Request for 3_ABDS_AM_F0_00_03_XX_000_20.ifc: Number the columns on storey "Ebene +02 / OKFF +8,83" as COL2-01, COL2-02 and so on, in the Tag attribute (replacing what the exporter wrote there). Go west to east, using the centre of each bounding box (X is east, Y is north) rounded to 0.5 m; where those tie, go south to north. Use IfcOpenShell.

First a look at what the model holds.

```python
import ifcopenshell
import ifcopenshell.util.element
import ifcopenshell.util.placement

model = ifcopenshell.open("3_ABDS_AM_F0_00_03_XX_000_20.ifc")
print(model.schema)
storey = next(s for s in model.by_type("IfcBuildingStorey") if s.Name == "Ebene +02 / OKFF +8,83")
columns = [e for e in ifcopenshell.util.element.get_decomposition(storey) if e.is_a("IfcColumn")]
for e in sorted(columns, key=lambda e: e.id()):
    origin = ifcopenshell.util.placement.get_local_placement(e.ObjectPlacement)[:3, 3]
    print(e.id(), e.Tag, e.Name, origin.round(2) + 0.0, sep=" | ")
```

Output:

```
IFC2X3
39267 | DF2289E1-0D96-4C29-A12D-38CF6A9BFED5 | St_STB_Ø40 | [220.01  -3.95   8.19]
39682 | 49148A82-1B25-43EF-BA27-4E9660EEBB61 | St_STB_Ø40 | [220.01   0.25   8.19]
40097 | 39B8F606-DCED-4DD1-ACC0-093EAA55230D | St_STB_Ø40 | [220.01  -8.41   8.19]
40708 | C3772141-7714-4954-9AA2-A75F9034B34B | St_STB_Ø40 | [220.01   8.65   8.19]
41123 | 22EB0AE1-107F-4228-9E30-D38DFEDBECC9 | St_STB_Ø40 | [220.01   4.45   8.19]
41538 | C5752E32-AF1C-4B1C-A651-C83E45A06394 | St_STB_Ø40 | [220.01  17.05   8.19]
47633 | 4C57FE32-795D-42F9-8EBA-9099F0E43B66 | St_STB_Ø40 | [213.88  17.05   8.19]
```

```python
import ifcopenshell
import ifcopenshell.geom
import ifcopenshell.util.element
import ifcopenshell.util.shape

model = ifcopenshell.open("3_ABDS_AM_F0_00_03_XX_000_20.ifc")
settings = ifcopenshell.geom.settings()
settings.set("use-world-coords", True)


def centre(element):
    shape = ifcopenshell.geom.create_shape(settings, element)
    return ifcopenshell.util.shape.get_bbox_centroid(shape.geometry)


storey = next(s for s in model.by_type("IfcBuildingStorey") if s.Name == "Ebene +02 / OKFF +8,83")
columns = [e for e in ifcopenshell.util.element.get_decomposition(storey) if e.is_a("IfcColumn")]

# Insertion points can sit at a corner or the storey origin, so sort by the geometry (in metres).
centres = {e: centre(e) for e in columns}
columns.sort(key=lambda e: (round(centres[e][0] / 0.5), centres[e][1]))

for i, e in enumerate(columns, start=1):
    number = f"COL2-{i:02d}"
    e.Tag = number
    print(e.id(), number)

model.write("3_ABDS_AM_F0_00_03_XX_000_20_updated.ifc")
```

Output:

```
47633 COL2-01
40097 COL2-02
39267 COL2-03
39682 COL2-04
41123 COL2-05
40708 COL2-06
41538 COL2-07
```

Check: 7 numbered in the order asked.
